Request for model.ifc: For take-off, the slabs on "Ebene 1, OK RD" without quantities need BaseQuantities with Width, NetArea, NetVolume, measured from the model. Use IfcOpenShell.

First a look at what the model holds.

```python
import ifcopenshell
import ifcopenshell.util.element
import ifcopenshell.util.unit

model = ifcopenshell.open("model.ifc")
print(model.schema)
for unit_type in ("LENGTHUNIT", "AREAUNIT", "VOLUMEUNIT"):
    print(unit_type, ifcopenshell.util.unit.calculate_unit_scale(model, unit_type))
storey = next(s for s in model.by_type("IfcBuildingStorey") if s.Name == "Ebene 1, OK RD")
slabs = [e for e in ifcopenshell.util.element.get_decomposition(storey) if e.is_a("IfcSlab")]
for e in sorted(slabs, key=lambda e: e.id()):
    print(e.id(), e.is_a(), e.Name, list(ifcopenshell.util.element.get_psets(e, qtos_only=True)), sep=" | ")
```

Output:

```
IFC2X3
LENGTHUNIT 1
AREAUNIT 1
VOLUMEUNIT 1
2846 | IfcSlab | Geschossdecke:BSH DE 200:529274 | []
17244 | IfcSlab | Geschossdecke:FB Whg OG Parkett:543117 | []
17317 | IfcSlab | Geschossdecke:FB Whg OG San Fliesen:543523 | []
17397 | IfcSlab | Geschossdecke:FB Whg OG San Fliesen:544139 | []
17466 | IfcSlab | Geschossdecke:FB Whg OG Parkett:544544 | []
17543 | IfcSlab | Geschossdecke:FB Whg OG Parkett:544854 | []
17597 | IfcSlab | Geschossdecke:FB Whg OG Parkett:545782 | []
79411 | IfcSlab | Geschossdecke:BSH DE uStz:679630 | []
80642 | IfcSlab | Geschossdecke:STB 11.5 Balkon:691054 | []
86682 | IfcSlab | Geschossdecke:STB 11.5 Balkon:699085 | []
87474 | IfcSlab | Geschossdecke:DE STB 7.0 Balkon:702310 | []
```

```python
import ifcopenshell
import ifcopenshell.api.pset
import ifcopenshell.geom
import ifcopenshell.util.element
import ifcopenshell.util.shape
import ifcopenshell.util.unit

model = ifcopenshell.open("model.ifc")
unit_scale = ifcopenshell.util.unit.calculate_unit_scale(model)
area_scale = ifcopenshell.util.unit.calculate_unit_scale(model, "AREAUNIT")
volume_scale = ifcopenshell.util.unit.calculate_unit_scale(model, "VOLUMEUNIT")
settings = ifcopenshell.geom.settings()

storey = next(s for s in model.by_type("IfcBuildingStorey") if s.Name == "Ebene 1, OK RD")
slabs = [e for e in ifcopenshell.util.element.get_decomposition(storey) if e.is_a("IfcSlab")]

for e in sorted(slabs, key=lambda e: e.id()):
    if ifcopenshell.util.element.get_psets(e, qtos_only=True, should_inherit=False):
        continue
    # Geometry comes back in metres, in the element's own axes.
    shape = ifcopenshell.geom.create_shape(settings, e)
    values = {
        "Width": ifcopenshell.util.shape.get_z(shape.geometry) / unit_scale,
        "NetArea": ifcopenshell.util.shape.get_footprint_area(shape.geometry) / area_scale,
        "NetVolume": ifcopenshell.util.shape.get_volume(shape.geometry) / volume_scale,
    }
    qto = ifcopenshell.api.pset.add_qto(model, product=e, name="BaseQuantities")
    ifcopenshell.api.pset.edit_qto(model, qto=qto, properties=values)
    print(e.id(), {k: round(v, 3) for k, v in values.items()})

model.write("model_edited.ifc")
```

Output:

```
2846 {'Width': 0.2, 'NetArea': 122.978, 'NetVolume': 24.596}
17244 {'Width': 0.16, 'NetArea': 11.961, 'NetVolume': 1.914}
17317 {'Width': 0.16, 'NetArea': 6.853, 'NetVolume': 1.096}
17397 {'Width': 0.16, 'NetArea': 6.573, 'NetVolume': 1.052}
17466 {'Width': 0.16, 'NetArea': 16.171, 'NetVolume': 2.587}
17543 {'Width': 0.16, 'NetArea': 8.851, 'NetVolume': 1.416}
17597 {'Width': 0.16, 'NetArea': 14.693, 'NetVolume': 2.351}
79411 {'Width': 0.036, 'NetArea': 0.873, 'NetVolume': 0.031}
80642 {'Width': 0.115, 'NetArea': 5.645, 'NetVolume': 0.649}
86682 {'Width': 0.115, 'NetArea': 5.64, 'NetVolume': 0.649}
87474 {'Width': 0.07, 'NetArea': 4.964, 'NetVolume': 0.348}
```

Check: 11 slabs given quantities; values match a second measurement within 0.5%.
